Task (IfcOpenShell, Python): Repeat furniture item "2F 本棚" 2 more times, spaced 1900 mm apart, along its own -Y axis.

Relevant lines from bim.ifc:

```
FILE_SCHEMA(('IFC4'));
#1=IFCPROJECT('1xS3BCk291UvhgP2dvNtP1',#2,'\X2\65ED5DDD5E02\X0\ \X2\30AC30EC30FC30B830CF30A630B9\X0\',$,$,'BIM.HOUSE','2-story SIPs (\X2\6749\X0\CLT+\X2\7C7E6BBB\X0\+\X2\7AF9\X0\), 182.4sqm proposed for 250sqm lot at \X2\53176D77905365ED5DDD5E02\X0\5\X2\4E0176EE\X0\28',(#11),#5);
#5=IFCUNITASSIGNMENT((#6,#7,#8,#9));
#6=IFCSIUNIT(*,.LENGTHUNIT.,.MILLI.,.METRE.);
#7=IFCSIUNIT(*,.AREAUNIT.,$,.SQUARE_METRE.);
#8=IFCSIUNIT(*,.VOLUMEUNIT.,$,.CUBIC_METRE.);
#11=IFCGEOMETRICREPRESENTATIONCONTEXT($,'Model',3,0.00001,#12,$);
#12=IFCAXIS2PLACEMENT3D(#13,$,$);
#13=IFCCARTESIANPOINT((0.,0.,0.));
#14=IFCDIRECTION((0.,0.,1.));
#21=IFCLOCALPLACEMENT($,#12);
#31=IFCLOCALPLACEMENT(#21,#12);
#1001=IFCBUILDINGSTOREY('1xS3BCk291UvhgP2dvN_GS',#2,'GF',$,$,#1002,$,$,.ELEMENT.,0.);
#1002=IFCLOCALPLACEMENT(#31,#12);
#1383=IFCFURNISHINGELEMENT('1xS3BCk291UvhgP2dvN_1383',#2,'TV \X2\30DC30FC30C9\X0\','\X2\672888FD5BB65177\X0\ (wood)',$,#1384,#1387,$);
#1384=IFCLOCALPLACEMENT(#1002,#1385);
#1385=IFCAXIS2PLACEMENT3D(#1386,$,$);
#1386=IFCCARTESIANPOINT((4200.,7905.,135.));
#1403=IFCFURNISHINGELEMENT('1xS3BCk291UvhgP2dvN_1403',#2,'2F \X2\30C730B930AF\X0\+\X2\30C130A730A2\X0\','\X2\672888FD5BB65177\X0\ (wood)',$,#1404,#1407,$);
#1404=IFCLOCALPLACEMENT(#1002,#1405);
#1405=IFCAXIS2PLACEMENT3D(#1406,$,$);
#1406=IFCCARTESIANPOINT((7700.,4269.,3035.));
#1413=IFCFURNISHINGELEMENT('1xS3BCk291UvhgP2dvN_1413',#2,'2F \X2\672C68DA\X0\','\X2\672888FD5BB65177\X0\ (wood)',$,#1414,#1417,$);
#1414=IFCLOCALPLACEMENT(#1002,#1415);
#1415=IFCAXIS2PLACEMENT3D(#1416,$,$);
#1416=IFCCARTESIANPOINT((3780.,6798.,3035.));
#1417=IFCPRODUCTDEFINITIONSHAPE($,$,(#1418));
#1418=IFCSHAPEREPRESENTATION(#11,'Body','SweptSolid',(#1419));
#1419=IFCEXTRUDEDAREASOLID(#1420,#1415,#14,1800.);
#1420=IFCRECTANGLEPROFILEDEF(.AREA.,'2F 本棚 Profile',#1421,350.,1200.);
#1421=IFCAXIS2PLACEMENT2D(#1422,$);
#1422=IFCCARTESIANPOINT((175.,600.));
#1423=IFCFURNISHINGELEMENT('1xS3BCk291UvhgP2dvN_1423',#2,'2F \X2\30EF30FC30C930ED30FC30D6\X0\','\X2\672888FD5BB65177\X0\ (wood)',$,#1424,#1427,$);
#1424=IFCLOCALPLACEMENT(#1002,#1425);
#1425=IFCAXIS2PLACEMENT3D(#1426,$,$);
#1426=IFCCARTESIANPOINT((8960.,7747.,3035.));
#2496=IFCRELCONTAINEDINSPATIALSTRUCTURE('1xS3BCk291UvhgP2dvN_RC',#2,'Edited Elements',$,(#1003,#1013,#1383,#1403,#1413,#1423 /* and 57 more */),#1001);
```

```python
import ifcopenshell
import ifcopenshell.api.geometry
import ifcopenshell.api.root
import ifcopenshell.util.element
import ifcopenshell.util.placement

model = ifcopenshell.open("bim.ifc")


def reuse_history(source, copy):
    """copy_class also copies each property set's owner history, people and application; keep the originals."""
    for rel in copy.IsDefinedBy:
        if rel.is_a("IfcRelDefinesByProperties") and (history := rel.RelatingPropertyDefinition.OwnerHistory):
            rel.RelatingPropertyDefinition.OwnerHistory = source.OwnerHistory
            ifcopenshell.util.element.remove_deep2(model, history)


source = model.by_guid("1xS3BCk291UvhgP2dvN_1413")
base = ifcopenshell.util.placement.get_local_placement(source.ObjectPlacement)
step = -base[:3, 1] * 1900.0

for i in range(1, 3):
    copy = ifcopenshell.api.root.copy_class(model, product=source)
    copy.Representation = ifcopenshell.util.element.copy_deep(
        model, source.Representation, exclude=["IfcGeometricRepresentationContext", "IfcRepresentationMap"]
    )
    reuse_history(source, copy)
    matrix = base.copy()
    matrix[:3, 3] += i * step
    print("added at", matrix[:3, 3].round(3) + 0.0)
    ifcopenshell.api.geometry.edit_object_placement(model, product=copy, matrix=matrix, is_si=False)

model.write("bim_rev.ifc")
```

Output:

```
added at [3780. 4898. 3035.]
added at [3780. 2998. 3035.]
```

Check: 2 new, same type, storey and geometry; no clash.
